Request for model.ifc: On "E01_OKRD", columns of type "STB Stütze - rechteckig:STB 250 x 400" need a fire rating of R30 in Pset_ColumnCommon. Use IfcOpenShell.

First a look at what the model holds.

```python
import ifcopenshell
import ifcopenshell.util.element

model = ifcopenshell.open("model.ifc")
print(model.schema)
storey = next(s for s in model.by_type("IfcBuildingStorey") if s.Name == "E01_OKRD")
columns = [e for e in ifcopenshell.util.element.get_decomposition(storey) if e.is_a("IfcColumn")]
seen = {}
for e in columns:
    element_type = ifcopenshell.util.element.get_type(e)
    key = (element_type.Name if element_type != e and element_type else None, ifcopenshell.util.element.get_pset(e, "Pset_ColumnCommon", "FireRating"))
    seen[key] = seen.get(key, 0) + 1
for (name, value), count in sorted(seen.items(), key=str):
    print(count, "x", name, "|", value)
```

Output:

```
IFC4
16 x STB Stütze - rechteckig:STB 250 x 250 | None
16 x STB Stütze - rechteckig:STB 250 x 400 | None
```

```python
import ifcopenshell
import ifcopenshell.api.pset
import ifcopenshell.util.element

model = ifcopenshell.open("model.ifc")

storey = next(s for s in model.by_type("IfcBuildingStorey") if s.Name == "E01_OKRD")
columns = [e for e in ifcopenshell.util.element.get_decomposition(storey) if e.is_a("IfcColumn")]

count = 0
for e in columns:
    element_type = ifcopenshell.util.element.get_type(e)
    if element_type in (None, e) or element_type.Name != "STB Stütze - rechteckig:STB 250 x 400":
        continue
    # add_pset returns the element's existing set when there is one.
    pset = ifcopenshell.api.pset.add_pset(model, product=e, name="Pset_ColumnCommon")
    ifcopenshell.api.pset.edit_pset(model, pset=pset, properties={"FireRating": "R30"})
    count += 1

print(count, "columns updated")

model.write("model-out.ifc")
```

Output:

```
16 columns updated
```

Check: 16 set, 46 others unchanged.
